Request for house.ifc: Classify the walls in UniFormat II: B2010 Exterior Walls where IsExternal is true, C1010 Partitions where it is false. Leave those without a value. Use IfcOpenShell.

First a look at what the model holds.

```python
import ifcopenshell
import ifcopenshell.util.element

model = ifcopenshell.open("house.ifc")
print(model.schema)
print("classifications:", [c.Name for c in model.by_type("IfcClassification")])
values = [ifcopenshell.util.element.get_pset(e, "Pset_WallCommon", "IsExternal") for e in model.by_type("IfcWall")]
for value in (True, False, None):
    print("IsExternal", value, values.count(value))
```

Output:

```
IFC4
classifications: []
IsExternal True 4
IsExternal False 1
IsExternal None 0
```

```python
import ifcopenshell
import ifcopenshell.api.classification
import ifcopenshell.util.element

model = ifcopenshell.open("house.ifc")

system = ifcopenshell.api.classification.add_classification(model, classification="UniFormat II")

walls = model.by_type("IfcWall")
external = {e: ifcopenshell.util.element.get_pset(e, "Pset_WallCommon", "IsExternal") for e in walls}
for flag, code, name in ((True, "B2010", "Exterior Walls"), (False, "C1010", "Partitions")):
    products = [e for e in walls if external[e] is flag]
    ifcopenshell.api.classification.add_reference(
        model, products=products, classification=system, identification=code, name=name
    )
    print(code, len(products))

model.write("house_edited.ifc")
```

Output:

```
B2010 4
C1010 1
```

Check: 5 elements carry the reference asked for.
